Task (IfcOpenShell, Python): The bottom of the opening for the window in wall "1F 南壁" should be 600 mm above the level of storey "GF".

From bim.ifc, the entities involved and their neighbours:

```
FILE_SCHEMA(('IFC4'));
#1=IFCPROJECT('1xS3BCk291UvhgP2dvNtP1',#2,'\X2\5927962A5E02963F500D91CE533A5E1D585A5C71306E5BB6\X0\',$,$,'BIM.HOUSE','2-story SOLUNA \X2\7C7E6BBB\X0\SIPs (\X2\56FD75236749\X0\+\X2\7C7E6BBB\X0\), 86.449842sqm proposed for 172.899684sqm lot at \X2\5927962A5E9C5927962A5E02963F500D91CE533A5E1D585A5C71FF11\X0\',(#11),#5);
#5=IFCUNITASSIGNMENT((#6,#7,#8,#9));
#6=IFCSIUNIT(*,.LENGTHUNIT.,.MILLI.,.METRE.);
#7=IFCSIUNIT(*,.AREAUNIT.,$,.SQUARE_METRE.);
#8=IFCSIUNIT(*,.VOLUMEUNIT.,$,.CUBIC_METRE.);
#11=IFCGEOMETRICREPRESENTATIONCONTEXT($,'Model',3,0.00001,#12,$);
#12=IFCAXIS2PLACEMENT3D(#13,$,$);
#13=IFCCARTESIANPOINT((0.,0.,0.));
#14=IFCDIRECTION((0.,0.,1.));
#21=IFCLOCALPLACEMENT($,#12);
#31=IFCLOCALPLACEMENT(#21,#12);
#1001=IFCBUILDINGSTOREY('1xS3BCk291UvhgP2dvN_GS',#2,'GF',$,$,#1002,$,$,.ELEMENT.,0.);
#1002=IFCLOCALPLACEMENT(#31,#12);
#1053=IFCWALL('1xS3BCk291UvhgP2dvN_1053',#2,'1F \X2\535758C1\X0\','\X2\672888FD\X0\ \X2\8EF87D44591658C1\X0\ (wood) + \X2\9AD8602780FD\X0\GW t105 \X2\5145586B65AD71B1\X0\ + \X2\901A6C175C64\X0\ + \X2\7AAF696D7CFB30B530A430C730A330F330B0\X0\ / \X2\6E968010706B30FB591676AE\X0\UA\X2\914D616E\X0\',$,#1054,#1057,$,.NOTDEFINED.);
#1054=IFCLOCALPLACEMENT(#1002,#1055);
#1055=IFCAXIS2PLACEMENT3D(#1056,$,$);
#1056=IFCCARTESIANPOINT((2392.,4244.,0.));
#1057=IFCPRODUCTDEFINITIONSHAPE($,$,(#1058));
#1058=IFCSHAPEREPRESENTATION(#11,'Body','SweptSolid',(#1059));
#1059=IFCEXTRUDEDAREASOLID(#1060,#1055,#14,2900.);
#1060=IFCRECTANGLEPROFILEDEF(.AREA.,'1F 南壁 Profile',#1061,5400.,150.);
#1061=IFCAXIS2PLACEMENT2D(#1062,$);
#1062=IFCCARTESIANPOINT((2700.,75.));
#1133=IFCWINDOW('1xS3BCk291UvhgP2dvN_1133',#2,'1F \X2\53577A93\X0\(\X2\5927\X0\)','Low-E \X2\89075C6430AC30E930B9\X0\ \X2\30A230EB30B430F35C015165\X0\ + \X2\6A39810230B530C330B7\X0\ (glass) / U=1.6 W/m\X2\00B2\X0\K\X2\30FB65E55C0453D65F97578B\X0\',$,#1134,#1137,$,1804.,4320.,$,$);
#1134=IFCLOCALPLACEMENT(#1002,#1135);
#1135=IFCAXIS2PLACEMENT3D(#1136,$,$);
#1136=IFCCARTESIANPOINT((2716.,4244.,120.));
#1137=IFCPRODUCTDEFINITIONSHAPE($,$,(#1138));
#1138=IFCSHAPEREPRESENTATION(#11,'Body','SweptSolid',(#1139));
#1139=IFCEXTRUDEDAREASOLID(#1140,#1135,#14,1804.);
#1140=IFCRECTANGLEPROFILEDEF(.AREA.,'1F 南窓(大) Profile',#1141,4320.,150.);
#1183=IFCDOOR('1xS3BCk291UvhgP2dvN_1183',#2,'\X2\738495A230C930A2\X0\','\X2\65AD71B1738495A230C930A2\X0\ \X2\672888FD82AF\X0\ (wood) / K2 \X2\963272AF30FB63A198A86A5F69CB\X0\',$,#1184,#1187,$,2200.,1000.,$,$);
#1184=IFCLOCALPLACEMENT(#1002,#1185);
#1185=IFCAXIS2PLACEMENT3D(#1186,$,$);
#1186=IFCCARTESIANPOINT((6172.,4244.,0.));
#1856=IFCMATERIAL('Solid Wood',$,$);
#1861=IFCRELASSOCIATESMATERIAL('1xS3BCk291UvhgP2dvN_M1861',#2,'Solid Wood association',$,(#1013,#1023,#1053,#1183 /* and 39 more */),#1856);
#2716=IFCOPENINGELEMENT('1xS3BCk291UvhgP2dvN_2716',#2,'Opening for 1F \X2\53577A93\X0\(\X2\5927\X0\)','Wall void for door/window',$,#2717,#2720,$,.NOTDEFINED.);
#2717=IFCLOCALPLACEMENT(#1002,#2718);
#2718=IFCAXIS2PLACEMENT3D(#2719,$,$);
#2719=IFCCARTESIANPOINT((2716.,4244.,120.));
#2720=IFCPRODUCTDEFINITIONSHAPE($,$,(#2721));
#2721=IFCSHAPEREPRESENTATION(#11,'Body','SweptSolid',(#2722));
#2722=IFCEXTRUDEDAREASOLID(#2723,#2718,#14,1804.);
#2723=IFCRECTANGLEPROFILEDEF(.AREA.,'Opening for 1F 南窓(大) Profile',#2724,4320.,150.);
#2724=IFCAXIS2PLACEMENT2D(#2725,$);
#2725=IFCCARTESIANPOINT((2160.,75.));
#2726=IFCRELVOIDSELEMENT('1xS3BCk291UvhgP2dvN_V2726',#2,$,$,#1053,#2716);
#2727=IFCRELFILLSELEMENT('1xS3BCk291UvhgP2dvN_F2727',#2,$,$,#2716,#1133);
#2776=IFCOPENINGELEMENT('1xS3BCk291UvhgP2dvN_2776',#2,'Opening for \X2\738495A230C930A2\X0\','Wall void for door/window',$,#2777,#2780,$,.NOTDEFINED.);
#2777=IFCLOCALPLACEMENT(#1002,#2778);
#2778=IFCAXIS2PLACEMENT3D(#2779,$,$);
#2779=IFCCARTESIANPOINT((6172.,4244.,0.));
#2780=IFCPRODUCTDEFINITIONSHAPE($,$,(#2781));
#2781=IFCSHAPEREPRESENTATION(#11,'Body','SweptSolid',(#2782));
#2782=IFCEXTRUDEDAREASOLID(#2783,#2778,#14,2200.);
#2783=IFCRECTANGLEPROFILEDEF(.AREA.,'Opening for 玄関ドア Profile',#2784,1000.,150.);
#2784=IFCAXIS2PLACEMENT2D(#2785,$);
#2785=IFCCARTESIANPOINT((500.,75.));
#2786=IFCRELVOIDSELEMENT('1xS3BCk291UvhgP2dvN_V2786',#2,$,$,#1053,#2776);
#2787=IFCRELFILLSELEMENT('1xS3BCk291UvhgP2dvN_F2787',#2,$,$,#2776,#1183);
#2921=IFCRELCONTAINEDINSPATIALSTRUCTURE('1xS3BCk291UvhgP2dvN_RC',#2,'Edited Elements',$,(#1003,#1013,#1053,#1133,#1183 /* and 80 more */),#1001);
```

```python
import numpy as np
import ifcopenshell
import ifcopenshell.api.geometry
import ifcopenshell.geom
import ifcopenshell.util.element
import ifcopenshell.util.placement
import ifcopenshell.util.shape
import ifcopenshell.util.unit

model = ifcopenshell.open("bim.ifc")
unit_scale = ifcopenshell.util.unit.calculate_unit_scale(model)

window = model.by_guid("1xS3BCk291UvhgP2dvN_1133")
opening = window.FillsVoids[0].RelatingOpeningElement
storey = ifcopenshell.util.element.get_container(window, ifc_class="IfcBuildingStorey")
level = ifcopenshell.util.placement.get_local_placement(storey.ObjectPlacement)[2, 3]

# The opening's origin need not be at the sill, so measure its lowest point.
shape = ifcopenshell.geom.create_shape(ifcopenshell.geom.settings(), opening)
bottom = ifcopenshell.util.shape.get_shape_bottom_elevation(shape, shape.geometry) / unit_scale
dz = level + 0.6 / unit_scale - bottom

shift = np.array([0.0, 0.0, dz])
# The window is not placed relative to its opening, so move both.
for product in (opening, window):
    matrix = ifcopenshell.util.placement.get_local_placement(product.ObjectPlacement)
    matrix[:3, 3] += shift
    ifcopenshell.api.geometry.edit_object_placement(model, product=product, matrix=matrix, is_si=False)

print(f"moved by {dz * unit_scale:+.3f} m")

model.write("bim_rev.ifc")
```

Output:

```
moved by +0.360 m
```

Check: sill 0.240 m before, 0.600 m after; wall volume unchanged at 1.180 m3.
